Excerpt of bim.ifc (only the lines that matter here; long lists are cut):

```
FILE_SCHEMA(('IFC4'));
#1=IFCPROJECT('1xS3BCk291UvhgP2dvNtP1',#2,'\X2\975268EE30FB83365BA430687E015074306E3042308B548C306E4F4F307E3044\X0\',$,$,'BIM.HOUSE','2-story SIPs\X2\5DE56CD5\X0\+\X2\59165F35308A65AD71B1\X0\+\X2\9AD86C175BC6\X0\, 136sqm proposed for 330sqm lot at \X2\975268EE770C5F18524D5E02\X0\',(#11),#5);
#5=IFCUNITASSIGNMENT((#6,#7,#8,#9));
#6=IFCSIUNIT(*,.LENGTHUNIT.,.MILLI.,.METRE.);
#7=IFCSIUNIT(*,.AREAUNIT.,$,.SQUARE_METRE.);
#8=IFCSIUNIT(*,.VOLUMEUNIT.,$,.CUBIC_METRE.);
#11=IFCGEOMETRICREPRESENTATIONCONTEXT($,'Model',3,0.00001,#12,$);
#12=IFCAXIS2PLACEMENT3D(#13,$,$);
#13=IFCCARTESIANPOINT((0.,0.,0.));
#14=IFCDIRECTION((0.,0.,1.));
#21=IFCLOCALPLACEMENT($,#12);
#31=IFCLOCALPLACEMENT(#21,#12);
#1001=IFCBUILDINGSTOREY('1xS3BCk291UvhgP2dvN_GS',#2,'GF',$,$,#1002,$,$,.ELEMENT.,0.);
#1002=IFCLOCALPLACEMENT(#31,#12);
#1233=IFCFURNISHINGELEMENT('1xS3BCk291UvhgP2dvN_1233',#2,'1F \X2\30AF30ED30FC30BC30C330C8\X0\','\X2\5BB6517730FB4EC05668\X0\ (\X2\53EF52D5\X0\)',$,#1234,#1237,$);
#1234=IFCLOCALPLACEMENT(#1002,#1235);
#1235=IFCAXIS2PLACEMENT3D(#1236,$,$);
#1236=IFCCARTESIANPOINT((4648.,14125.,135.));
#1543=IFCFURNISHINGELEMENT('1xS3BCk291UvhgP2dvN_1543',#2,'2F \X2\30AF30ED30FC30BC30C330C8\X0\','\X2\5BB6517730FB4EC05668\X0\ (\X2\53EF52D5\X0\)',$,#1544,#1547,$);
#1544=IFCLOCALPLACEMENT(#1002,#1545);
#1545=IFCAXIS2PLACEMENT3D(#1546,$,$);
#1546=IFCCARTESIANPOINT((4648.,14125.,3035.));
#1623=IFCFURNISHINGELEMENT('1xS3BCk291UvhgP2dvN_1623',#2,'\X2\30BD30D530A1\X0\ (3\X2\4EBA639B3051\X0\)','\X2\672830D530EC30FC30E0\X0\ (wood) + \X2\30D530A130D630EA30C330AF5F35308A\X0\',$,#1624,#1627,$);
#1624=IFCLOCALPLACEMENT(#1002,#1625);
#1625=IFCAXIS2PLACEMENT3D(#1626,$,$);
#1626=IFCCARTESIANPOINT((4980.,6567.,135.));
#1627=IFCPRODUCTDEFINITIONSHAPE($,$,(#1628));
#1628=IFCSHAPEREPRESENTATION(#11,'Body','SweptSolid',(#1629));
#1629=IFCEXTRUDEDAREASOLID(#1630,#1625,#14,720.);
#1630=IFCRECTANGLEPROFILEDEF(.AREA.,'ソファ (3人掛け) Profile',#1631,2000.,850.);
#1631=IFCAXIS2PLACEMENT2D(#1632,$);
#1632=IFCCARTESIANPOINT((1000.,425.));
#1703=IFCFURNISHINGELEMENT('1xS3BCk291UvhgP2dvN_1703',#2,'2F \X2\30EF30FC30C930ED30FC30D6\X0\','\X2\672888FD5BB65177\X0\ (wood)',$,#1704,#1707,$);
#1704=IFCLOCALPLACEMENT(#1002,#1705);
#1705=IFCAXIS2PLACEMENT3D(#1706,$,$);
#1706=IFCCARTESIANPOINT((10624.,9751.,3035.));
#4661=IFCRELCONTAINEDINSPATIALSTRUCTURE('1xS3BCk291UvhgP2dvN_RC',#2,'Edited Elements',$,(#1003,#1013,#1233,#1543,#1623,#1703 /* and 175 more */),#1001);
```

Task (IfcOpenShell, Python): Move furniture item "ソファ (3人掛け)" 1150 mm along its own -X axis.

```python
import ifcopenshell
import ifcopenshell.api.geometry
import ifcopenshell.util.placement

model = ifcopenshell.open("bim.ifc")

item = model.by_guid("1xS3BCk291UvhgP2dvN_1623")
matrix = ifcopenshell.util.placement.get_local_placement(item.ObjectPlacement)
matrix[:3, 3] -= matrix[:3, 0] * 1150.0
ifcopenshell.api.geometry.edit_object_placement(model, product=item, matrix=matrix, is_si=False)

print(ifcopenshell.util.placement.get_local_placement(item.ObjectPlacement).round(3) + 0.0)

model.write("bim_updated.ifc")
```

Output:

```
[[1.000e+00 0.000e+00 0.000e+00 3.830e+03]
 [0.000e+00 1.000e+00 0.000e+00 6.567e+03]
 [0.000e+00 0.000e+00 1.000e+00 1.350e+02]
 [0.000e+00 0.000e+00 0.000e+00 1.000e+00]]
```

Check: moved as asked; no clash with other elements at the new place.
